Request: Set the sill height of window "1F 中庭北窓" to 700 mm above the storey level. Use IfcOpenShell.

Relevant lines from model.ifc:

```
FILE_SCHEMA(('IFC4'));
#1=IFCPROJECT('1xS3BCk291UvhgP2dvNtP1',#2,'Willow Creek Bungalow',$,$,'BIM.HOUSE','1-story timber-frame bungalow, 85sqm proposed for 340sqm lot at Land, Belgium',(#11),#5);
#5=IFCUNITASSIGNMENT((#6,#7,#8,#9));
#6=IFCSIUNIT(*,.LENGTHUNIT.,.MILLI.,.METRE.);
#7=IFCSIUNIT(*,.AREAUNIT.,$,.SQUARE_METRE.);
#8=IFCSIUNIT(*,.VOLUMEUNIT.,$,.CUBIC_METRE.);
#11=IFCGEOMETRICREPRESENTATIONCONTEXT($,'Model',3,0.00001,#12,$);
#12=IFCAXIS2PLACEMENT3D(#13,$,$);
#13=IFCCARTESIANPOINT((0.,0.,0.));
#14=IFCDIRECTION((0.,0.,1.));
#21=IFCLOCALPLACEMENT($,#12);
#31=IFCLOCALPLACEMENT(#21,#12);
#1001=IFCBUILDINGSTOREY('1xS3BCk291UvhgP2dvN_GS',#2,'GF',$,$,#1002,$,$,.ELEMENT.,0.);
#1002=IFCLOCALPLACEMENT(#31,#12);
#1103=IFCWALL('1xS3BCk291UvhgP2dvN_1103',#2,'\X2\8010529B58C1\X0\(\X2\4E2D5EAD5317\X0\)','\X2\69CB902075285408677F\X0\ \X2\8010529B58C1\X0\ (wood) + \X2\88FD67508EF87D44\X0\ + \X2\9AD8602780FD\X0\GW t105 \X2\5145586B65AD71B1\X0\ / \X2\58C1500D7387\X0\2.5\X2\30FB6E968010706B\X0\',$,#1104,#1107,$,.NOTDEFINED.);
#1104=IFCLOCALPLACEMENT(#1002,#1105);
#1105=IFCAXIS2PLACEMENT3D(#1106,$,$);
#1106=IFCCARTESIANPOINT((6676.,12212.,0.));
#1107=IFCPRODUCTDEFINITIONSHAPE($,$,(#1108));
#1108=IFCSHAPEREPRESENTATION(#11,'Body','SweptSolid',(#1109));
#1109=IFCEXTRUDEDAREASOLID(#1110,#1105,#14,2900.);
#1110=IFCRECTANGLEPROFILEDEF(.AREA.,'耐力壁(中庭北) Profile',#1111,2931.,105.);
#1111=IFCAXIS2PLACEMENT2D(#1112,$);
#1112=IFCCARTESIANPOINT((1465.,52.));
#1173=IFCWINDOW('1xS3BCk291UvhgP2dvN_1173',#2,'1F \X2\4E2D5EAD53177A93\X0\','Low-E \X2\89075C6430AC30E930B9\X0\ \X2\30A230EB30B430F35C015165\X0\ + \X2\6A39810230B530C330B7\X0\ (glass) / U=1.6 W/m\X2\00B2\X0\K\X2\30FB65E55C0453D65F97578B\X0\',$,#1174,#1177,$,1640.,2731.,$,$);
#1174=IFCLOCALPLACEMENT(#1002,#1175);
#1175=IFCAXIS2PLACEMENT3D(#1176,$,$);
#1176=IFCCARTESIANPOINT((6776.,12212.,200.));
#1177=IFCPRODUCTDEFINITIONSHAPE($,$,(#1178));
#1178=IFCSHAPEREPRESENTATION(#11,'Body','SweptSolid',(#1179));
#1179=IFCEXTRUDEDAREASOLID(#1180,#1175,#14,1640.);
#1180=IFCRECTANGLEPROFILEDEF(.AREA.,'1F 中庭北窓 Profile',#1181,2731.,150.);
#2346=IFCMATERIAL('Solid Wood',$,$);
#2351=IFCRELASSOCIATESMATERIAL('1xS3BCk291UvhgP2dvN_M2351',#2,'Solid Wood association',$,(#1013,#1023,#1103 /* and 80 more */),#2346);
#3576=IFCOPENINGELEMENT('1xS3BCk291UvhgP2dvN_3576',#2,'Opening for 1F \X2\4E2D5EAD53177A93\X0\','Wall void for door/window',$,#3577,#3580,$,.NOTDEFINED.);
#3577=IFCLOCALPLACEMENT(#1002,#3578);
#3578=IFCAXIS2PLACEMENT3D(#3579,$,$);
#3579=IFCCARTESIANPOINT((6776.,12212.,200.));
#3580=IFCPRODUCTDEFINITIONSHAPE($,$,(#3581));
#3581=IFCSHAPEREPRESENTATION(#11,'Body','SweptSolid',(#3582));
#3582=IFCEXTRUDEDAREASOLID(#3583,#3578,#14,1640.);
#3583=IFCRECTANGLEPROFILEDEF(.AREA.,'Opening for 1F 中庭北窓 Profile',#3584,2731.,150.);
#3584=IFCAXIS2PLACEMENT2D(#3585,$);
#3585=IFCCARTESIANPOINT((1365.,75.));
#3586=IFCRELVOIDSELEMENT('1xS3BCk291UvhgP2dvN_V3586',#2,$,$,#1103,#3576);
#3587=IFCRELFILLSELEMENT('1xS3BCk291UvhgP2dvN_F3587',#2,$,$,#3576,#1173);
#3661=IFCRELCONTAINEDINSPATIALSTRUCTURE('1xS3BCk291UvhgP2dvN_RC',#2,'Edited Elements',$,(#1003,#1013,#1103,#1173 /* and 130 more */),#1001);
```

```python
import numpy as np
import ifcopenshell
import ifcopenshell.api.geometry
import ifcopenshell.geom
import ifcopenshell.util.element
import ifcopenshell.util.placement
import ifcopenshell.util.shape
import ifcopenshell.util.unit

model = ifcopenshell.open("model.ifc")
unit_scale = ifcopenshell.util.unit.calculate_unit_scale(model)

window = model.by_guid("1xS3BCk291UvhgP2dvN_1173")
opening = window.FillsVoids[0].RelatingOpeningElement
storey = ifcopenshell.util.element.get_container(window, ifc_class="IfcBuildingStorey")
level = ifcopenshell.util.placement.get_local_placement(storey.ObjectPlacement)[2, 3]

# The opening's origin need not be at the sill, so measure its lowest point.
shape = ifcopenshell.geom.create_shape(ifcopenshell.geom.settings(), opening)
bottom = ifcopenshell.util.shape.get_shape_bottom_elevation(shape, shape.geometry) / unit_scale
dz = level + 700.0 - bottom

shift = np.array([0.0, 0.0, dz])
# The window is not placed relative to its opening, so move both.
for product in (opening, window):
    matrix = ifcopenshell.util.placement.get_local_placement(product.ObjectPlacement)
    matrix[:3, 3] += shift
    ifcopenshell.api.geometry.edit_object_placement(model, product=product, matrix=matrix, is_si=False)

print(f"moved by {dz * unit_scale:+.3f} m")

model.write("model_updated.ifc")
```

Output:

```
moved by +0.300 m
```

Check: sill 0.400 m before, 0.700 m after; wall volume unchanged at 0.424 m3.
